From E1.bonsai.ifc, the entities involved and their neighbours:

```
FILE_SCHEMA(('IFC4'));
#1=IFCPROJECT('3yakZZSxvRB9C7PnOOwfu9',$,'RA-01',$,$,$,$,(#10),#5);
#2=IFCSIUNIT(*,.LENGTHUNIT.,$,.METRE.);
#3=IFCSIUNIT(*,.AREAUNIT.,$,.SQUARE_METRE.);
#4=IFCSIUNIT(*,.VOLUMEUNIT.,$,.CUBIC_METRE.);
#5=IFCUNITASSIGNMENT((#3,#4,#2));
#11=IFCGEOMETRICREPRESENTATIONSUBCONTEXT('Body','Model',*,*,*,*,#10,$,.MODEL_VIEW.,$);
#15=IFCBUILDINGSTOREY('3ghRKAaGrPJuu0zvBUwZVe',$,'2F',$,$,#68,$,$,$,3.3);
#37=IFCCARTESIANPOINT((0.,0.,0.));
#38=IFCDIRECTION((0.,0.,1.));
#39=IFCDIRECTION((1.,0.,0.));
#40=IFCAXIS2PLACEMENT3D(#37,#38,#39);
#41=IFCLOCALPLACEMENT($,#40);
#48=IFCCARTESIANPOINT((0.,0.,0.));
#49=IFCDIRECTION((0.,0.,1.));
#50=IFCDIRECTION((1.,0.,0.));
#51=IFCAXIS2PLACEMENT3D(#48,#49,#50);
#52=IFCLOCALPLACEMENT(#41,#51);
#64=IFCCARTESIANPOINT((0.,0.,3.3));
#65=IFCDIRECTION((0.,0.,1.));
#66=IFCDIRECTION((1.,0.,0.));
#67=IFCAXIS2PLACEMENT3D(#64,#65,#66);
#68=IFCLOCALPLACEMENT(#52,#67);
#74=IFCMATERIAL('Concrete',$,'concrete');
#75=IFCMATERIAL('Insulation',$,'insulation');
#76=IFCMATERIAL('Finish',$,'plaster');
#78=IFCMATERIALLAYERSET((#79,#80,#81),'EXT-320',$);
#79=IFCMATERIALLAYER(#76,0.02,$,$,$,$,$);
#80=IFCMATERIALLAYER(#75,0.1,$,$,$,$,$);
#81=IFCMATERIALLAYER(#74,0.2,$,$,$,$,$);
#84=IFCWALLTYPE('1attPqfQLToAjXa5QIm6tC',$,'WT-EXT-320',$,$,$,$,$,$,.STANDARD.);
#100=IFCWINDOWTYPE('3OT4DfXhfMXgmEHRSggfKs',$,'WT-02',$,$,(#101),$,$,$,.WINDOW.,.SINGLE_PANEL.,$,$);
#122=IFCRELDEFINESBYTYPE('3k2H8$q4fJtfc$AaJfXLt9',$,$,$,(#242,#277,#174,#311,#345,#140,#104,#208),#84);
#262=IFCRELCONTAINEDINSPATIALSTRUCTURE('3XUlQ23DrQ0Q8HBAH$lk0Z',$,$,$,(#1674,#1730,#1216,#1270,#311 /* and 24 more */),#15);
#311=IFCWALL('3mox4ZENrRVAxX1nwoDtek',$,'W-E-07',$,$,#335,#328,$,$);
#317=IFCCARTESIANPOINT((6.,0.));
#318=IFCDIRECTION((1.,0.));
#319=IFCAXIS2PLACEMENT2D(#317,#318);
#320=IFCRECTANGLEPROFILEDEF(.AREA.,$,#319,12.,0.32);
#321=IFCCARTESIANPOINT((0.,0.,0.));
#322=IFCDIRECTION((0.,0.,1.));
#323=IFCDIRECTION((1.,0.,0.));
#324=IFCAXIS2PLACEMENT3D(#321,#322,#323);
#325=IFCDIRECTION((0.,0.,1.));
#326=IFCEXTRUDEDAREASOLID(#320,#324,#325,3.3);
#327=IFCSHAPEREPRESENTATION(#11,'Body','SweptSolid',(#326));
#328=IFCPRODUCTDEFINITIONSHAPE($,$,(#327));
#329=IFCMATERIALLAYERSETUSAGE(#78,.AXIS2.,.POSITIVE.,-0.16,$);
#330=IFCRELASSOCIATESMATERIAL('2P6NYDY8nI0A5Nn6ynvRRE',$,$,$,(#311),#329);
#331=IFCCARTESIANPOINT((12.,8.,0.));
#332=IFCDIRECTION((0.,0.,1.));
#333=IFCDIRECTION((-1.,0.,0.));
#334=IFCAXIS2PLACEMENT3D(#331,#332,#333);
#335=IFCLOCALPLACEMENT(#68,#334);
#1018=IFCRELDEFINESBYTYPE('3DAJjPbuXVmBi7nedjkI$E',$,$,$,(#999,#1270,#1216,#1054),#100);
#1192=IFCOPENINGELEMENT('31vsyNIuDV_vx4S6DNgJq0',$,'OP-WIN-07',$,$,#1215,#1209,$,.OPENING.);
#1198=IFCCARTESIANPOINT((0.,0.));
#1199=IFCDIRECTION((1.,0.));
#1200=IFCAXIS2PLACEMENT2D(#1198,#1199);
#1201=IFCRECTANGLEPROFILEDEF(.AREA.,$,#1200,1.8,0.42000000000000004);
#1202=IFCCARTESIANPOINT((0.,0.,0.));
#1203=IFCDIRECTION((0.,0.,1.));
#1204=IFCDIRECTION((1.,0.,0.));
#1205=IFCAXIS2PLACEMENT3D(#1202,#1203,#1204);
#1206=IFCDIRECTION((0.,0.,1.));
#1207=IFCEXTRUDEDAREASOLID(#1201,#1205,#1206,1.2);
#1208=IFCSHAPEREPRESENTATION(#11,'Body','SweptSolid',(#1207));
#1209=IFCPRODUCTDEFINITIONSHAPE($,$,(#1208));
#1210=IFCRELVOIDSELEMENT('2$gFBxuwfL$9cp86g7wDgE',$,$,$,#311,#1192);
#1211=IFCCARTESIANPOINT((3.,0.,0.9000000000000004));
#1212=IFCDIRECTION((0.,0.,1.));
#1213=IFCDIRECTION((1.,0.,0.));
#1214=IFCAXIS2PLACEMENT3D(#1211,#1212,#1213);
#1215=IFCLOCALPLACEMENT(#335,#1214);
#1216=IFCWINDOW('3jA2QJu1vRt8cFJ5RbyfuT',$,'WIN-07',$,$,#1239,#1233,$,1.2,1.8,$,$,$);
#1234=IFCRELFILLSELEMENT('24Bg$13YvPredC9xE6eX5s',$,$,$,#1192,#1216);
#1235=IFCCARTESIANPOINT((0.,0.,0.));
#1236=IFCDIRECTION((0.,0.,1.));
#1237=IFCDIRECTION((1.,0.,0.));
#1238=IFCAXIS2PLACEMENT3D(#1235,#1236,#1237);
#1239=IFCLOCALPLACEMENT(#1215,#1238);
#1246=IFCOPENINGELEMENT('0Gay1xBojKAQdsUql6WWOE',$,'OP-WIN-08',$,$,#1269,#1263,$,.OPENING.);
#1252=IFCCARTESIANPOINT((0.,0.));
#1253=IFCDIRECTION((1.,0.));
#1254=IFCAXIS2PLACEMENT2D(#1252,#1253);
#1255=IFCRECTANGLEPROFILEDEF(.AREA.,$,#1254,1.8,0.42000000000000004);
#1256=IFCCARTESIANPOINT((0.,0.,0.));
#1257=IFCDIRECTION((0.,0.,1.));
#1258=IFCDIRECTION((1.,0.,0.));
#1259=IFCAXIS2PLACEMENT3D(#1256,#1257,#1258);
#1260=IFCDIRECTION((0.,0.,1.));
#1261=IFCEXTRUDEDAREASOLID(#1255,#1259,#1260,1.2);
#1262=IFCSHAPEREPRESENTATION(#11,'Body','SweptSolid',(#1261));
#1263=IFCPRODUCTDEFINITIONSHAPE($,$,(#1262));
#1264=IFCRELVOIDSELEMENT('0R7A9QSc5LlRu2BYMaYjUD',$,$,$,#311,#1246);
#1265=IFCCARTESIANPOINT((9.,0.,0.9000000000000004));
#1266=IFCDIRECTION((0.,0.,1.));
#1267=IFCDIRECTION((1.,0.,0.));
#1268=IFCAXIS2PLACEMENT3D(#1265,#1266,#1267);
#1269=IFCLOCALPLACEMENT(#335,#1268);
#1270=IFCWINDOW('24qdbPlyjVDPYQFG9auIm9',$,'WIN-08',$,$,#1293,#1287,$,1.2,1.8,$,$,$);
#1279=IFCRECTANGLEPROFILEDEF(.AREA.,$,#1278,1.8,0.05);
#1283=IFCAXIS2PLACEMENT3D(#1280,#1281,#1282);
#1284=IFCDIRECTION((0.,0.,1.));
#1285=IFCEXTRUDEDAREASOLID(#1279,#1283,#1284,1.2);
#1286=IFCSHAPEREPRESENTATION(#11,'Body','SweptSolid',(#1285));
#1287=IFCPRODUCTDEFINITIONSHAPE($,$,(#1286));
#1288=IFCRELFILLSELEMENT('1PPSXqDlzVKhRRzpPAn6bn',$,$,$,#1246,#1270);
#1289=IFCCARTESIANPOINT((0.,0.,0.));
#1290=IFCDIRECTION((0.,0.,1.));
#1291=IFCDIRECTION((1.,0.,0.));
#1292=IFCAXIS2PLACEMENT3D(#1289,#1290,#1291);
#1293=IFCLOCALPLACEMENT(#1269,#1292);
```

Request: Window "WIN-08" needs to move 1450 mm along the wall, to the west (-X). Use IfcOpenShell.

```python
import ifcopenshell
import ifcopenshell.api.geometry
import ifcopenshell.util.placement
import ifcopenshell.util.unit

model = ifcopenshell.open("E1.bonsai.ifc")
unit_scale = ifcopenshell.util.unit.calculate_unit_scale(model)

window = model.by_id(1270)
opening = window.FillsVoids[0].RelatingOpeningElement
wall = opening.VoidsElements[0].RelatingBuildingElement

wall_matrix = ifcopenshell.util.placement.get_local_placement(wall.ObjectPlacement)
shift = wall_matrix[:3, 0] * 1.45 / unit_scale
before = ifcopenshell.util.placement.get_local_placement(window.ObjectPlacement)[:3, 3].copy()

# The window is placed relative to its opening, so it follows when the opening moves.
matrix = ifcopenshell.util.placement.get_local_placement(opening.ObjectPlacement)
matrix[:3, 3] += shift
ifcopenshell.api.geometry.edit_object_placement(
    model, product=opening, matrix=matrix, is_si=False, should_transform_children=True
)

after = ifcopenshell.util.placement.get_local_placement(window.ObjectPlacement)[:3, 3]
print("window moved by", (after - before).round(3) + 0.0)

model.write("E1.bonsai_rev.ifc")
```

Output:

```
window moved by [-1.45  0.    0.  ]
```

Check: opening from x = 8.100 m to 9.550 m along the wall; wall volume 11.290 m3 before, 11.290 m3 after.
